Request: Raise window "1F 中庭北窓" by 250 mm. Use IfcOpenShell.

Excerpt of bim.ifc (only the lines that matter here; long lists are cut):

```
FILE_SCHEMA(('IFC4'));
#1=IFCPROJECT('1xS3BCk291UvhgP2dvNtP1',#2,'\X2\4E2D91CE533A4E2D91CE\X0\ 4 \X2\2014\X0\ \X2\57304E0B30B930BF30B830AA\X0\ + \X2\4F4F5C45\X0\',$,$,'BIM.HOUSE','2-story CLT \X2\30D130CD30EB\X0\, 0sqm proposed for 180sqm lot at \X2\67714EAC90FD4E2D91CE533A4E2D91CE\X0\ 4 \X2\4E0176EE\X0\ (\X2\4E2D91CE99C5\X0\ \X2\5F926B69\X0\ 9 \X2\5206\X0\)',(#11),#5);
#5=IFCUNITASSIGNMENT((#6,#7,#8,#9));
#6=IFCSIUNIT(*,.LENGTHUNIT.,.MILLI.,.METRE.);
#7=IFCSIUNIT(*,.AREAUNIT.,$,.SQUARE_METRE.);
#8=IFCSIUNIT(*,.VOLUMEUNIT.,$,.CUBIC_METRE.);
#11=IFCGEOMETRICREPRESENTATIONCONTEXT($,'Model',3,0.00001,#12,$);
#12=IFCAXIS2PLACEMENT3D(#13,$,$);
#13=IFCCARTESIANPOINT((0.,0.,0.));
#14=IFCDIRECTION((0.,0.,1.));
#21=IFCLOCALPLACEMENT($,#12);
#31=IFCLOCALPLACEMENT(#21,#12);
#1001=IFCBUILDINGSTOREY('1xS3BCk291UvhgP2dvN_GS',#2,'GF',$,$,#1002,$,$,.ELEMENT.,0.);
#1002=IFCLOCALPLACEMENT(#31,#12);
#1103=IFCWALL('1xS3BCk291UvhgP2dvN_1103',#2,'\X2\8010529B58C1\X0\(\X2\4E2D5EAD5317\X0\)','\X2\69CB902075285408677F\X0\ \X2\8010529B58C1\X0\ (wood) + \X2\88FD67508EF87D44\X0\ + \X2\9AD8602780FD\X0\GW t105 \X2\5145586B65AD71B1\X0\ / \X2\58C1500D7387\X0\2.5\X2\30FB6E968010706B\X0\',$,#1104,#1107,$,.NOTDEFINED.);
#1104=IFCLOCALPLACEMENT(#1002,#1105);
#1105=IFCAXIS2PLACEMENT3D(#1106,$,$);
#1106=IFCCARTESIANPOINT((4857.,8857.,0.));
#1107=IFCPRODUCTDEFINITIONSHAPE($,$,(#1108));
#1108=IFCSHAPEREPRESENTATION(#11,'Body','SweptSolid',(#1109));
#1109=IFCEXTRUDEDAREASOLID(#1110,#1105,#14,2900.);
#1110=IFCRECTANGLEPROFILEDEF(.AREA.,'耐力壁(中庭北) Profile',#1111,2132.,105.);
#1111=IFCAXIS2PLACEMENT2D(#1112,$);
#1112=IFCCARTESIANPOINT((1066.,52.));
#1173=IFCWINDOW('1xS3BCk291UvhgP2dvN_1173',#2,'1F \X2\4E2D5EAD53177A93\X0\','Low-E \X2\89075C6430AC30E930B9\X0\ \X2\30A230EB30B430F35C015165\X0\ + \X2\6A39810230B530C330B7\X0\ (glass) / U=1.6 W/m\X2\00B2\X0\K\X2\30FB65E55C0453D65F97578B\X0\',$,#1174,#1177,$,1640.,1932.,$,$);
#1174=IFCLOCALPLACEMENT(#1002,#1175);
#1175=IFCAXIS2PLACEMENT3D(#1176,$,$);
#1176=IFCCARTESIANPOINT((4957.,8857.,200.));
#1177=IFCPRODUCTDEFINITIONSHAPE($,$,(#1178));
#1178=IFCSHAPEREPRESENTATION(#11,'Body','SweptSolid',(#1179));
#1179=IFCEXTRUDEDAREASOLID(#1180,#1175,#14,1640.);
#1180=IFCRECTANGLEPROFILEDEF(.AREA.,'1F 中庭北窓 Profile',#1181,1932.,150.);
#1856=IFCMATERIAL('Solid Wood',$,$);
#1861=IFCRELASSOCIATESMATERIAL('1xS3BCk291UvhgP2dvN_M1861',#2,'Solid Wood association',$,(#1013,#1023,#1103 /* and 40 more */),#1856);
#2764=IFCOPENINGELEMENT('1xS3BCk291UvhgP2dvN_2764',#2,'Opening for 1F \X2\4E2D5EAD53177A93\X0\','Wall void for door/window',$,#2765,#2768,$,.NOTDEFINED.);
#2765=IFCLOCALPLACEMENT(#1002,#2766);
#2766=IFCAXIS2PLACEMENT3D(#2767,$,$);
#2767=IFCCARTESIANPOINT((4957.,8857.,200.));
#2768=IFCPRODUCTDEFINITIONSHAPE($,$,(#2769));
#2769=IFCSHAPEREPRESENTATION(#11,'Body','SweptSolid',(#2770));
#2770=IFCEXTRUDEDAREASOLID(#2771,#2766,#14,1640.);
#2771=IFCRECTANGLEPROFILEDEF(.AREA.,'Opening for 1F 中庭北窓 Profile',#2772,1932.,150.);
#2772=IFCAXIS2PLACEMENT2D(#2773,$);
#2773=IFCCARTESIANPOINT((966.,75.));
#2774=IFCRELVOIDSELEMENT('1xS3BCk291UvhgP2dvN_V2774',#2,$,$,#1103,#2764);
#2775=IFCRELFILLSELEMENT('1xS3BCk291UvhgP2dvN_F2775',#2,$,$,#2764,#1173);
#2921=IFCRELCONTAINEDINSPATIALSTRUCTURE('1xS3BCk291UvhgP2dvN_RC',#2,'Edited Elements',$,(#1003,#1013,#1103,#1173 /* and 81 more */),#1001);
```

```python
import numpy as np
import ifcopenshell
import ifcopenshell.api.geometry
import ifcopenshell.util.placement
import ifcopenshell.util.unit

model = ifcopenshell.open("bim.ifc")
unit_scale = ifcopenshell.util.unit.calculate_unit_scale(model)

window = model.by_guid("1xS3BCk291UvhgP2dvN_1173")
opening = window.FillsVoids[0].RelatingOpeningElement
dz = 250.0

shift = np.array([0.0, 0.0, dz])
# The window is not placed relative to its opening, so move both.
for product in (opening, window):
    matrix = ifcopenshell.util.placement.get_local_placement(product.ObjectPlacement)
    matrix[:3, 3] += shift
    ifcopenshell.api.geometry.edit_object_placement(model, product=product, matrix=matrix, is_si=False)

print(f"moved by {dz * unit_scale:+.3f} m")

model.write("bim_updated.ifc")
```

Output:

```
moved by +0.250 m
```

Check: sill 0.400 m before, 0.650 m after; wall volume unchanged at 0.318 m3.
